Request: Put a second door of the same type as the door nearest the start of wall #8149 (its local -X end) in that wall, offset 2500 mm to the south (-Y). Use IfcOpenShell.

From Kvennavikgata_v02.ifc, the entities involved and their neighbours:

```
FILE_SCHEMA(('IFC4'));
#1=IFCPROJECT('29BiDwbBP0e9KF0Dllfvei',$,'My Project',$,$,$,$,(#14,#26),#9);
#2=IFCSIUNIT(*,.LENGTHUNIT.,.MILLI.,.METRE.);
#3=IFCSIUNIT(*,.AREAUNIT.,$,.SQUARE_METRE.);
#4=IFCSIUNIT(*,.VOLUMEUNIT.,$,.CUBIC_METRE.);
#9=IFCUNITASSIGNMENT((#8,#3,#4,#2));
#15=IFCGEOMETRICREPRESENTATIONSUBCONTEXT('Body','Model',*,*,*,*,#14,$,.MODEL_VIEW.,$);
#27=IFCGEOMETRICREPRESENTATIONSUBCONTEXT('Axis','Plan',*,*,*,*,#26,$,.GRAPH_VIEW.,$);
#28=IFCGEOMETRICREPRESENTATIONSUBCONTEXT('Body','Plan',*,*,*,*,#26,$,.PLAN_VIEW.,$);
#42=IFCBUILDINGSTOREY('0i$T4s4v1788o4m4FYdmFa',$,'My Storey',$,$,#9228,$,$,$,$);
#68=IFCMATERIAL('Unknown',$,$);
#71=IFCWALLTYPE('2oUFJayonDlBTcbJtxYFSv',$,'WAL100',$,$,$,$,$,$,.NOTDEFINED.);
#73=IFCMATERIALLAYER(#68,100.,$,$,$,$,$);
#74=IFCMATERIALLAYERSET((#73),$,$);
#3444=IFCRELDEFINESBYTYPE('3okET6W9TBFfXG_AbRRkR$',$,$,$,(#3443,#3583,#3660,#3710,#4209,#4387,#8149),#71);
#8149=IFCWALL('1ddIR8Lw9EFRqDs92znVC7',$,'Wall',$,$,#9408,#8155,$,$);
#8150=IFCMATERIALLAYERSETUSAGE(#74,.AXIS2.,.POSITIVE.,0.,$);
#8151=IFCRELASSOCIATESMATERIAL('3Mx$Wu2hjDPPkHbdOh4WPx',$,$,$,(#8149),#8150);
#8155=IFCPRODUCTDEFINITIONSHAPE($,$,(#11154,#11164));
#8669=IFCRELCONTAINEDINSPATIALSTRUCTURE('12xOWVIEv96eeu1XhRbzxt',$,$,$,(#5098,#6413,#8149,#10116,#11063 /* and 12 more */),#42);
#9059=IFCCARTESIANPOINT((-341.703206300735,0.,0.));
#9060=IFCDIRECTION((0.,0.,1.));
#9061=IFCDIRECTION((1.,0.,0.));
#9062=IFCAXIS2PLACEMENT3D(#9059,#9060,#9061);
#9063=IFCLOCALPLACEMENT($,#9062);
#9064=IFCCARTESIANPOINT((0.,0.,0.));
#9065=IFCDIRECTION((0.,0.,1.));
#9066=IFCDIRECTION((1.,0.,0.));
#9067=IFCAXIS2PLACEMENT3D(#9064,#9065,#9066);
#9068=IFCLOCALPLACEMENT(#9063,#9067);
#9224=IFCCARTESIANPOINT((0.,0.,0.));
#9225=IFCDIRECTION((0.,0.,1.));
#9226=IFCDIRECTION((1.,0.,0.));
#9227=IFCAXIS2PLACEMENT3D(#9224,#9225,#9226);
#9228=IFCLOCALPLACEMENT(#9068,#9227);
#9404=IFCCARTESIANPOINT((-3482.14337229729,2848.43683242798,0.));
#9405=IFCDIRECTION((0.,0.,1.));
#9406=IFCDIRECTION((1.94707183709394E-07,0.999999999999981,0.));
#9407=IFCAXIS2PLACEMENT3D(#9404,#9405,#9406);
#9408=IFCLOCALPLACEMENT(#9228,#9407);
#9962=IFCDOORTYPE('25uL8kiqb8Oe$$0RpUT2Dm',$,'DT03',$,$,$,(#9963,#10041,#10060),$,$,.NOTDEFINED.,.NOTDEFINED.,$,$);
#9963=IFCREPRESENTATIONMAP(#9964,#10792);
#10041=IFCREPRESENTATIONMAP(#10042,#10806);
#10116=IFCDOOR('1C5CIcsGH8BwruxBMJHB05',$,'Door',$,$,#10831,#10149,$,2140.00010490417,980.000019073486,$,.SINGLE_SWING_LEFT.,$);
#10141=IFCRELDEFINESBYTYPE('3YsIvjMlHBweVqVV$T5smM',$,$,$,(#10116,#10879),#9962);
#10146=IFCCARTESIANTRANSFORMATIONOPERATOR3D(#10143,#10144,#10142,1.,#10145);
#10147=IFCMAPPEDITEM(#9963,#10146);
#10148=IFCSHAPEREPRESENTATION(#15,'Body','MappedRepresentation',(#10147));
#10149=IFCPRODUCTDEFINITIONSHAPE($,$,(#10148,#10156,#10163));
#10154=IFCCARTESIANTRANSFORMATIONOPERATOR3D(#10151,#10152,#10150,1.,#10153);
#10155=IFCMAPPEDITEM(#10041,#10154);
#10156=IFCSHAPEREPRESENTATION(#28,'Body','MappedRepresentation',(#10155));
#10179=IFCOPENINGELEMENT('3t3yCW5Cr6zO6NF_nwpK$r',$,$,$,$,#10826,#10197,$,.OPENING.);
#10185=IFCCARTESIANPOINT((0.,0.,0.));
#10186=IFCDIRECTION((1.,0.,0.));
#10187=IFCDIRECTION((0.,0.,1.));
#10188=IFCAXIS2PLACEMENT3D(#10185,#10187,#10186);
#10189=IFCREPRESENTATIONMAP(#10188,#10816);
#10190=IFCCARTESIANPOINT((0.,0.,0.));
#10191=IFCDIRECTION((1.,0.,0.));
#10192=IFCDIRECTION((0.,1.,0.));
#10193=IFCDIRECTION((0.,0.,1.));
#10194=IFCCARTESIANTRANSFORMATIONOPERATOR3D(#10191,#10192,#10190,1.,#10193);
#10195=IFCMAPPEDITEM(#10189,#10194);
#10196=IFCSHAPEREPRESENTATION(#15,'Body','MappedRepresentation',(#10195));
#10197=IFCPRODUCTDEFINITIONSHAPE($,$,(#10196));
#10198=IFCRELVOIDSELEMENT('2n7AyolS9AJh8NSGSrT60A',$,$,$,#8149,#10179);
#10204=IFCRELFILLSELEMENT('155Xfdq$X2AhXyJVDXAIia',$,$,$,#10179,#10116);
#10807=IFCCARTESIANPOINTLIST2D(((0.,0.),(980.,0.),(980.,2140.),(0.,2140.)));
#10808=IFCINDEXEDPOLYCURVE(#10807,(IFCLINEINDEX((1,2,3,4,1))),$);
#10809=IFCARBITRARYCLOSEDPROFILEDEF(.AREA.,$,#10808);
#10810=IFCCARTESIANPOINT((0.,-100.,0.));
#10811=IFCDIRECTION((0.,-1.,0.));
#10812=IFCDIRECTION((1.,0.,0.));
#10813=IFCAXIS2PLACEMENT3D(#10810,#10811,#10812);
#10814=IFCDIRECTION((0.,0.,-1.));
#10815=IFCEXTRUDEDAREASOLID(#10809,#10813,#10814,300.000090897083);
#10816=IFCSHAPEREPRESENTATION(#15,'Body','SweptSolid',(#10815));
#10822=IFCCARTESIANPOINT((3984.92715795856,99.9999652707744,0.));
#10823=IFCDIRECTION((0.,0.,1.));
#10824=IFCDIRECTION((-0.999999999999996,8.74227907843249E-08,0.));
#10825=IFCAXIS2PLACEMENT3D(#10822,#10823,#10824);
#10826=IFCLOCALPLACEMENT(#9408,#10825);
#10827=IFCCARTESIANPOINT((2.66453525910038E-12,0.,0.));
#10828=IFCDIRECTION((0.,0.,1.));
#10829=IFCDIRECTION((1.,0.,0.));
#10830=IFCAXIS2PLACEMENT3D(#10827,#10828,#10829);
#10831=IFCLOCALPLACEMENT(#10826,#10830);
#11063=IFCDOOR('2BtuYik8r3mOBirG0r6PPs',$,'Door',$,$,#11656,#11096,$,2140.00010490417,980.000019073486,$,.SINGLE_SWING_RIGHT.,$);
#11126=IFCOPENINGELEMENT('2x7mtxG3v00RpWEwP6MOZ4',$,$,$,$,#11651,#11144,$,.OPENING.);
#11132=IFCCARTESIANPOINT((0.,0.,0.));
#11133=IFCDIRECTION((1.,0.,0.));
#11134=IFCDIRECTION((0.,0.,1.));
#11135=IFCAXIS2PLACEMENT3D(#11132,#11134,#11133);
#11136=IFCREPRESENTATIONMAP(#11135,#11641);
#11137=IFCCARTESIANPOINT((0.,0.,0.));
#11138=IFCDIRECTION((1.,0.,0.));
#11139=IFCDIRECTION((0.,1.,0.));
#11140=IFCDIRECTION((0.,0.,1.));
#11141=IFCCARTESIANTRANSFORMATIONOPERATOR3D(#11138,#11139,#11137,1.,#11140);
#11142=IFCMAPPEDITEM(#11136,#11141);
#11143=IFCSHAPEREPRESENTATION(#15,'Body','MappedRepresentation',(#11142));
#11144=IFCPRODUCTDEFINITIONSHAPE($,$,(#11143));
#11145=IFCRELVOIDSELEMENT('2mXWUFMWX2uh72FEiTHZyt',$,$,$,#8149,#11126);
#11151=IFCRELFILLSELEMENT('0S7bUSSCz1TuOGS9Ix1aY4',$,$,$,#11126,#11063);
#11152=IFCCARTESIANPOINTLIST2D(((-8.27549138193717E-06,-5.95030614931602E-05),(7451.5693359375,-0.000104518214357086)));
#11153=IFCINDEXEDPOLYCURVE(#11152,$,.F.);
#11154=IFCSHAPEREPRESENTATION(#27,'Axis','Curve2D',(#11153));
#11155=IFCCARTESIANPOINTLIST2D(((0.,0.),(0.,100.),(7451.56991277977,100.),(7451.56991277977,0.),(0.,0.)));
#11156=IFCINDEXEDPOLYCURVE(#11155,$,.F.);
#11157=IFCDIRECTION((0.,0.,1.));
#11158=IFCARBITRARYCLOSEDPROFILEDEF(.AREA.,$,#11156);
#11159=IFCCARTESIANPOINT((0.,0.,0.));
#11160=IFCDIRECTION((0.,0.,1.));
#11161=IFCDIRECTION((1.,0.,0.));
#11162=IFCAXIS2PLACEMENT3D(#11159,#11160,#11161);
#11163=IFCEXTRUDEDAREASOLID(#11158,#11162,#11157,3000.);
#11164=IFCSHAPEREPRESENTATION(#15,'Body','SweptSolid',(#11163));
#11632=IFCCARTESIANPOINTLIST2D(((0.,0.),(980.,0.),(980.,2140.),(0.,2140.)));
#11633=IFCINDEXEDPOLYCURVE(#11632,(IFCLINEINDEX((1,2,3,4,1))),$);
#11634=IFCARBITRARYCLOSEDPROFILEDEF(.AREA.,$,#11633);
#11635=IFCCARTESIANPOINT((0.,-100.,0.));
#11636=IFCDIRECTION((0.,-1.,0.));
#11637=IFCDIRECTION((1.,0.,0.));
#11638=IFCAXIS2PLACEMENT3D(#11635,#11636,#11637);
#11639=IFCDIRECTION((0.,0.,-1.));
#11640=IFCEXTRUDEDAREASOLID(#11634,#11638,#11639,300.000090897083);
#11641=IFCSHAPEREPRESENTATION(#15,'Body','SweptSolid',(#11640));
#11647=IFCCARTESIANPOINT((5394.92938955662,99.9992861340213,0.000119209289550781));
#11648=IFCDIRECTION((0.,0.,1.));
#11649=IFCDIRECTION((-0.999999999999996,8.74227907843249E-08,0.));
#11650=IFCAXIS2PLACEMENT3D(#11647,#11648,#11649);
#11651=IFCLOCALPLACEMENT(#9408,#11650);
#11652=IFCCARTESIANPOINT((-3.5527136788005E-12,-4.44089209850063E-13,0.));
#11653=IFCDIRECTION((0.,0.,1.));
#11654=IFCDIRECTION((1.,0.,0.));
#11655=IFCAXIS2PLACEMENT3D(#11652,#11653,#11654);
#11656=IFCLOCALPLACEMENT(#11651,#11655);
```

```python
import ifcopenshell
import ifcopenshell.api.feature
import ifcopenshell.api.geometry
import ifcopenshell.api.root
import ifcopenshell.geom
import ifcopenshell.util.element
import ifcopenshell.util.placement
import ifcopenshell.util.shape
import ifcopenshell.util.unit

model = ifcopenshell.open("Kvennavikgata_v02.ifc")
unit_scale = ifcopenshell.util.unit.calculate_unit_scale(model)
settings = ifcopenshell.geom.settings()


def volume(element):
    """Net volume in cubic metres, openings subtracted."""
    shape = ifcopenshell.geom.create_shape(settings, element)
    return ifcopenshell.util.shape.get_volume(shape.geometry)


door = model.by_guid("1C5CIcsGH8BwruxBMJHB05")
opening = door.FillsVoids[0].RelatingOpeningElement
wall = opening.VoidsElements[0].RelatingBuildingElement
before = volume(wall)
shift = ifcopenshell.util.placement.get_local_placement(wall.ObjectPlacement)[:3, 0] * -2.5 / unit_scale

# copy_class copies the void relationship, type, container and properties, but no geometry.
new_opening = ifcopenshell.api.root.copy_class(model, product=opening)
new_opening.Representation = ifcopenshell.util.element.copy_deep(
    model, opening.Representation, exclude=["IfcGeometricRepresentationContext", "IfcRepresentationMap"]
)
new_door = ifcopenshell.api.root.copy_class(model, product=door)
new_door.Representation = ifcopenshell.util.element.copy_deep(
    model, door.Representation, exclude=["IfcGeometricRepresentationContext", "IfcRepresentationMap"]
)
ifcopenshell.api.feature.add_filling(model, opening=new_opening, element=new_door)

for old, new in ((opening, new_opening), (door, new_door)):
    matrix = ifcopenshell.util.placement.get_local_placement(old.ObjectPlacement)
    matrix[:3, 3] += shift
    ifcopenshell.api.geometry.edit_object_placement(model, product=new, matrix=matrix, is_si=False)

after = volume(wall)

print(f"wall volume {before:.3f} -> {after:.3f} m3")

model.write("Kvennavikgata_v02_updated.ifc")
```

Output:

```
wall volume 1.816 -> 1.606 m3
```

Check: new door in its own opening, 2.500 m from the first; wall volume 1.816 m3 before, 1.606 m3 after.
